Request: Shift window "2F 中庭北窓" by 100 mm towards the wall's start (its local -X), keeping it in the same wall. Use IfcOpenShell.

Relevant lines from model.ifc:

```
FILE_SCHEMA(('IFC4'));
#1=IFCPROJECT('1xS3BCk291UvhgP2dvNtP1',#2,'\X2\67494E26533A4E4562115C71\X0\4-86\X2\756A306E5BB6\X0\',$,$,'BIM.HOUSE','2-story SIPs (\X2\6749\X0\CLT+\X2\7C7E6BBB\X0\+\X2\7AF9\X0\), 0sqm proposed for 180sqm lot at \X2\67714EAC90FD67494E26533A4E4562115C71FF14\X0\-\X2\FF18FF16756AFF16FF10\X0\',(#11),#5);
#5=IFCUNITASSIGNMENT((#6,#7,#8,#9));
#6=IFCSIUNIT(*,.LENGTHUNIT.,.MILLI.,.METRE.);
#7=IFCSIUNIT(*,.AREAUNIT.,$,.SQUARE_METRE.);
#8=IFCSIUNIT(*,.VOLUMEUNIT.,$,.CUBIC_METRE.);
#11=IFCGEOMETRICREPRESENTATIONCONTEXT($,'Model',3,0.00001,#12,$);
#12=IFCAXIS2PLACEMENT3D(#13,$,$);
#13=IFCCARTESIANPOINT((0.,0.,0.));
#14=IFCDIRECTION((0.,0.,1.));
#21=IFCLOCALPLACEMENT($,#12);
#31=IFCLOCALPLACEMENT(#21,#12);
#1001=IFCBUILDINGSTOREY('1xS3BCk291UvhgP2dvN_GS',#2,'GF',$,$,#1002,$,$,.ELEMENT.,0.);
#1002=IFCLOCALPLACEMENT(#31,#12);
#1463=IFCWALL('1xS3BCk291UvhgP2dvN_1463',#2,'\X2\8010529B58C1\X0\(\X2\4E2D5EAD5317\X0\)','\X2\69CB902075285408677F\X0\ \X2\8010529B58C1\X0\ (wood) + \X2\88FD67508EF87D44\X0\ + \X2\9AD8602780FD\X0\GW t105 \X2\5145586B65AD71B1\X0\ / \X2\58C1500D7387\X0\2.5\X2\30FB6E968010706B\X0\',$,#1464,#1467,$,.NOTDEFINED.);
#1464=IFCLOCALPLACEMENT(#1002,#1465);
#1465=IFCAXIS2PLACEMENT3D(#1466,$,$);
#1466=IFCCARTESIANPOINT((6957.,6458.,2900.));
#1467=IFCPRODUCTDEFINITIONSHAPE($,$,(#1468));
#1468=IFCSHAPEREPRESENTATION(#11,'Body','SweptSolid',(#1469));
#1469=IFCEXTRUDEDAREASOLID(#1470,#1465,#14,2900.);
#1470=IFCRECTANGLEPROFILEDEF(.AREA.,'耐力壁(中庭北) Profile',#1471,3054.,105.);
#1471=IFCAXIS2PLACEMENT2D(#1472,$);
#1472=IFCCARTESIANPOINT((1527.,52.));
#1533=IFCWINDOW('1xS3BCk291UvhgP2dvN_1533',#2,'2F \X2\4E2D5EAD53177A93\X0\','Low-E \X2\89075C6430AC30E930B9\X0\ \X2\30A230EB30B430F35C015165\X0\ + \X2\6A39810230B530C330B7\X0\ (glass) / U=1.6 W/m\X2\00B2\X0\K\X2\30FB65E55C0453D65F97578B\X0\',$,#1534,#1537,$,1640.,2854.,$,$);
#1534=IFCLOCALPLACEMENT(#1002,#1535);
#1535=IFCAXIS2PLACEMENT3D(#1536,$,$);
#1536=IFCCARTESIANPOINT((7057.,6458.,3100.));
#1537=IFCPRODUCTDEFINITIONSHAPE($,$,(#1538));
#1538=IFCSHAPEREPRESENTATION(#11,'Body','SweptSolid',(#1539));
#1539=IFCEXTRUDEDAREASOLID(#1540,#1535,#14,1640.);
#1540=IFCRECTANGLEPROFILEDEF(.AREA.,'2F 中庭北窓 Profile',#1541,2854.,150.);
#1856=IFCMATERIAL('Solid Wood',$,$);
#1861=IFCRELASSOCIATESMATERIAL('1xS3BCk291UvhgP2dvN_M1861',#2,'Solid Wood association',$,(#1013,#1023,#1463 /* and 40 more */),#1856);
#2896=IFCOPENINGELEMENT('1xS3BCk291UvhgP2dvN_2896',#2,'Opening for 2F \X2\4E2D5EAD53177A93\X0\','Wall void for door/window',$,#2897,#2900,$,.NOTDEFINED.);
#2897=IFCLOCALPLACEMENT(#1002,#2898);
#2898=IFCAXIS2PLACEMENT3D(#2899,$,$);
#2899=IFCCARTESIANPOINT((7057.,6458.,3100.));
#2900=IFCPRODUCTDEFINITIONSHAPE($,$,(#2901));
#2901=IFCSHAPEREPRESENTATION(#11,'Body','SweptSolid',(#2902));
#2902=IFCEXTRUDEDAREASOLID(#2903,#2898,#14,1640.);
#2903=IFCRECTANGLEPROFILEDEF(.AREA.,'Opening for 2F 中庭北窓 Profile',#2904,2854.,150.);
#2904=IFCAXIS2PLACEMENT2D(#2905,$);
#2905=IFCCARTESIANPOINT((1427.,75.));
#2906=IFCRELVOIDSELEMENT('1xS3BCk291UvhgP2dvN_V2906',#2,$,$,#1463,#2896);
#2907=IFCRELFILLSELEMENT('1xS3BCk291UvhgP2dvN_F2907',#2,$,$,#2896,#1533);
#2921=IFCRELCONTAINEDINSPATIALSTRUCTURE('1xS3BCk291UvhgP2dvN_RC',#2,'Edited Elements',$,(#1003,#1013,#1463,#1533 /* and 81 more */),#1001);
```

```python
import ifcopenshell
import ifcopenshell.api.geometry
import ifcopenshell.util.placement
import ifcopenshell.util.unit

model = ifcopenshell.open("model.ifc")
unit_scale = ifcopenshell.util.unit.calculate_unit_scale(model)

window = model.by_guid("1xS3BCk291UvhgP2dvN_1533")
opening = window.FillsVoids[0].RelatingOpeningElement
wall = opening.VoidsElements[0].RelatingBuildingElement

wall_matrix = ifcopenshell.util.placement.get_local_placement(wall.ObjectPlacement)
shift = wall_matrix[:3, 0] * -0.1 / unit_scale
before = ifcopenshell.util.placement.get_local_placement(window.ObjectPlacement)[:3, 3].copy()

# The window is not placed relative to its opening, so move both.
for product in (opening, window):
    matrix = ifcopenshell.util.placement.get_local_placement(product.ObjectPlacement)
    matrix[:3, 3] += shift
    ifcopenshell.api.geometry.edit_object_placement(model, product=product, matrix=matrix, is_si=False)

after = ifcopenshell.util.placement.get_local_placement(window.ObjectPlacement)[:3, 3]
print("window moved by", (after - before).round(3) + 0.0)

model.write("model_edited.ifc")
```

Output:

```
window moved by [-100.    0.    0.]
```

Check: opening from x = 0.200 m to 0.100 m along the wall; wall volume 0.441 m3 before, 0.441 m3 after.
